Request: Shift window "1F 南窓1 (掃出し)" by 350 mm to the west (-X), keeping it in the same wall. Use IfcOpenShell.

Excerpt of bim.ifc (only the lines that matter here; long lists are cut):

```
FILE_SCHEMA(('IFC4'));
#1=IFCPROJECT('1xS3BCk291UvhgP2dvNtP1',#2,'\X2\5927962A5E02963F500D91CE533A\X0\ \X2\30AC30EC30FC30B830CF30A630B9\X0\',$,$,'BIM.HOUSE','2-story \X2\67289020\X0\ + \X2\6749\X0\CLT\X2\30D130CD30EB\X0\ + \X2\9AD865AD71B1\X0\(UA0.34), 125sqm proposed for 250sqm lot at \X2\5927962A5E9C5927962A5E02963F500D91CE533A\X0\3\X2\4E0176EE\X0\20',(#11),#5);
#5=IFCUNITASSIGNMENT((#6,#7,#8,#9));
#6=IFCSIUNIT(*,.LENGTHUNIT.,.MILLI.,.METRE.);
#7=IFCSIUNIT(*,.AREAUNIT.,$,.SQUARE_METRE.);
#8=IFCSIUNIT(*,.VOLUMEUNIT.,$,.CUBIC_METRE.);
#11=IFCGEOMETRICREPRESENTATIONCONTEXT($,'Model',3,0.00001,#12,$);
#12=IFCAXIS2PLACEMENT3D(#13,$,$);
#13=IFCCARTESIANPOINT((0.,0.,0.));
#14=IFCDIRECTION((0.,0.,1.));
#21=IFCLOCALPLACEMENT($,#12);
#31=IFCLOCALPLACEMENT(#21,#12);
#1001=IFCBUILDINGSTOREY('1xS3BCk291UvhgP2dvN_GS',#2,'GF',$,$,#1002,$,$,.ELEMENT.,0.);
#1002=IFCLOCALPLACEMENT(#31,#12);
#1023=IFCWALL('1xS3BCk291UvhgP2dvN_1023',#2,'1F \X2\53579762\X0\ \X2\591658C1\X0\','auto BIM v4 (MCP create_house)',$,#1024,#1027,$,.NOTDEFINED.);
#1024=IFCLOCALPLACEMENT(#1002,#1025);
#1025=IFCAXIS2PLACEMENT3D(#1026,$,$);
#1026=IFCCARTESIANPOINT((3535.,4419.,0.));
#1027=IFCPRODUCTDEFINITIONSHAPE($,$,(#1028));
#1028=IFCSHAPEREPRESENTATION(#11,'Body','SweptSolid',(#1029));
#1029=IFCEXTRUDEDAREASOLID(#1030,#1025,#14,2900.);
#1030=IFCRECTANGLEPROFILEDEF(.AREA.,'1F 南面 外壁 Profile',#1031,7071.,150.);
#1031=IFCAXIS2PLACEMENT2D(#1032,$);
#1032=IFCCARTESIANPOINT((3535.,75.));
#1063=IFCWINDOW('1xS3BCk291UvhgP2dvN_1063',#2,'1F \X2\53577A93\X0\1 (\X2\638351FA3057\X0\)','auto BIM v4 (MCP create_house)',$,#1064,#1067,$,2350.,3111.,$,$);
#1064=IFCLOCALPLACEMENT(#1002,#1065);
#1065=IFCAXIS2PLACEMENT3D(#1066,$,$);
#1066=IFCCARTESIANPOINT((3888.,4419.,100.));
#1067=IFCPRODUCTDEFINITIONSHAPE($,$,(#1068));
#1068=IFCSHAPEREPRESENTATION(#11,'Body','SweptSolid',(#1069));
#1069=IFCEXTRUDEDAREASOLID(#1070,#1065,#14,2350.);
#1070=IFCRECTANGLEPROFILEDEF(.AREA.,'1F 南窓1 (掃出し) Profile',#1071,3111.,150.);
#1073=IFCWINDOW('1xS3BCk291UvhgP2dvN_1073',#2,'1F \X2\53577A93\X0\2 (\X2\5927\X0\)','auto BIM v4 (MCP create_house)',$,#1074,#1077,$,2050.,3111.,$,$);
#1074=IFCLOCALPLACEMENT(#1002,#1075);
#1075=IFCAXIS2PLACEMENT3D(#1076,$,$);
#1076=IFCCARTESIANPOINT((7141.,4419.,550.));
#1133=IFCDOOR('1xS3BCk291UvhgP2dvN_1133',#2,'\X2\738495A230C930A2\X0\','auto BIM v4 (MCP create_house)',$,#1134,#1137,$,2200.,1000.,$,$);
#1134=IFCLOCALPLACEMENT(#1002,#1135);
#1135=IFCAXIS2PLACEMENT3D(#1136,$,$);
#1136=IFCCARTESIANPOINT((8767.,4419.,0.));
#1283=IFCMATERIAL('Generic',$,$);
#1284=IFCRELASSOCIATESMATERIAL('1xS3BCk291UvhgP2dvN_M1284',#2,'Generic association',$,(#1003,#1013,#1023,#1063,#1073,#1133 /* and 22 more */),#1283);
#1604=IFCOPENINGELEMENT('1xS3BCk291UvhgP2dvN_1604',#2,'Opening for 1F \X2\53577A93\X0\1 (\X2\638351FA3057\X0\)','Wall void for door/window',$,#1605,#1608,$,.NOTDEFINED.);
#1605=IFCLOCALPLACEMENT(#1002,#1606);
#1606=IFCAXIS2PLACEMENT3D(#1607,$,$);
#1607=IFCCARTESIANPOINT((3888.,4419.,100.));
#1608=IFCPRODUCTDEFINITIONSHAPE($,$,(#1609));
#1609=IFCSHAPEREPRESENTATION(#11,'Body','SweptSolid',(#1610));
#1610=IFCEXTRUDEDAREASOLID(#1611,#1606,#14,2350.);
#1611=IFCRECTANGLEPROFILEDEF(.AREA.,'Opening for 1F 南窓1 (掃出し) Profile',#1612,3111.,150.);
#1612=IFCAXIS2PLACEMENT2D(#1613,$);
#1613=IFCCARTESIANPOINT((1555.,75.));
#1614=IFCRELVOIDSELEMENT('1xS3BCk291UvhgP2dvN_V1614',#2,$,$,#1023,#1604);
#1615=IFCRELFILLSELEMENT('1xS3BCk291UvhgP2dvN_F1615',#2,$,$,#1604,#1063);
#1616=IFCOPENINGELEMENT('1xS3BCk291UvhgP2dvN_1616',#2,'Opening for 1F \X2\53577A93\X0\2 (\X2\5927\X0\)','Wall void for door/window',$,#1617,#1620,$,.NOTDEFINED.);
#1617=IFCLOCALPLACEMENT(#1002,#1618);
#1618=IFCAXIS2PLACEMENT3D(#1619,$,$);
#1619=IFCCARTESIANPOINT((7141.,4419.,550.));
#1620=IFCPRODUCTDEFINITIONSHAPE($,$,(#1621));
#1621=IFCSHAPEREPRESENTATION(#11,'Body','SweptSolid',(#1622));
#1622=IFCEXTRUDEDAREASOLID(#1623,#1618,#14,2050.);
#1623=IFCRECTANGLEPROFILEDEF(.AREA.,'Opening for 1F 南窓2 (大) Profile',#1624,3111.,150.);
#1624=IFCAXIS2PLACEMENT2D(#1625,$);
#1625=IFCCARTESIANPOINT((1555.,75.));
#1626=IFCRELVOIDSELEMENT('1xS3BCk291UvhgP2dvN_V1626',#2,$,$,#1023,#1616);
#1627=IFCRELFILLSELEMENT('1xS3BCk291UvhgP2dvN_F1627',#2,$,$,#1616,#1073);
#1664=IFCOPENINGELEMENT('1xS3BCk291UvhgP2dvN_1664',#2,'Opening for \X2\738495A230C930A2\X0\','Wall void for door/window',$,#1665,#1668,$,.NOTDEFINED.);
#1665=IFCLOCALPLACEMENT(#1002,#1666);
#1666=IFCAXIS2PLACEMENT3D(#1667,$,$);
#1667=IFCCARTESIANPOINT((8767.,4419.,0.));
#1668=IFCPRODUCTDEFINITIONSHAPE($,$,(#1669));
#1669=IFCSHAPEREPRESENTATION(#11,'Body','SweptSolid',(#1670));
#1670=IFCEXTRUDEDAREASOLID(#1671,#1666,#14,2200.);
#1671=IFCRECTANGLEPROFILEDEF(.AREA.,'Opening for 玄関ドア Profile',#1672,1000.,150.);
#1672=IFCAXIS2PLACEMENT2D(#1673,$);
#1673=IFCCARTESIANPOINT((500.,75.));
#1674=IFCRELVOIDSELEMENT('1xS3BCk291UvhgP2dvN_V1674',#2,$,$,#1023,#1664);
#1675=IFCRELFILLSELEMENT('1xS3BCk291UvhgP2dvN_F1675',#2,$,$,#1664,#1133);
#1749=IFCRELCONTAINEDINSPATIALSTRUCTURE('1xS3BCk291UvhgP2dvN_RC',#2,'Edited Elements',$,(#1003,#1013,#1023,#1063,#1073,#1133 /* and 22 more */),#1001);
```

```python
import ifcopenshell
import ifcopenshell.api.geometry
import ifcopenshell.util.placement
import ifcopenshell.util.unit

model = ifcopenshell.open("bim.ifc")
unit_scale = ifcopenshell.util.unit.calculate_unit_scale(model)

window = model.by_guid("1xS3BCk291UvhgP2dvN_1063")
opening = window.FillsVoids[0].RelatingOpeningElement
wall = opening.VoidsElements[0].RelatingBuildingElement

wall_matrix = ifcopenshell.util.placement.get_local_placement(wall.ObjectPlacement)
shift = wall_matrix[:3, 0] * -0.35 / unit_scale
before = ifcopenshell.util.placement.get_local_placement(window.ObjectPlacement)[:3, 3].copy()

# The window is not placed relative to its opening, so move both.
for product in (opening, window):
    matrix = ifcopenshell.util.placement.get_local_placement(product.ObjectPlacement)
    matrix[:3, 3] += shift
    ifcopenshell.api.geometry.edit_object_placement(model, product=product, matrix=matrix, is_si=False)

after = ifcopenshell.util.placement.get_local_placement(window.ObjectPlacement)[:3, 3]
print("window moved by", (after - before).round(3) + 0.0)

model.write("bim_v2.ifc")
```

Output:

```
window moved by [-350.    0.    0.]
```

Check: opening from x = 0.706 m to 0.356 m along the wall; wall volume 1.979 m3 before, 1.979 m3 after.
